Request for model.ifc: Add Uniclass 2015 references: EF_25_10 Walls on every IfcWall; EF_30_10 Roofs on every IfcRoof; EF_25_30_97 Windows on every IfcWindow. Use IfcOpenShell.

First a look at what the model holds.

```python
import ifcopenshell

model = ifcopenshell.open("model.ifc")
print(model.schema)
print("classifications:", [c.Name for c in model.by_type("IfcClassification")])
for ifc_class in ("IfcDoor", "IfcRoof", "IfcStair", "IfcWall", "IfcWindow"):
    print(ifc_class, len(model.by_type(ifc_class)))
```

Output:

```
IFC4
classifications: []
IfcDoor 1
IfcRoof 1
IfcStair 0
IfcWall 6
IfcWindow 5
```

```python
import ifcopenshell
import ifcopenshell.api.classification

model = ifcopenshell.open("model.ifc")

system = ifcopenshell.api.classification.add_classification(model, classification="Uniclass 2015")

codes = {
    "IfcWall": ("EF_25_10", "Walls"),
    "IfcRoof": ("EF_30_10", "Roofs"),
    "IfcWindow": ("EF_25_30_97", "Windows"),
}
for ifc_class, (code, name) in codes.items():
    products = model.by_type(ifc_class)
    ifcopenshell.api.classification.add_reference(
        model, products=products, classification=system, identification=code, name=name
    )
    print(code, len(products))

model.write("model_edited.ifc")
```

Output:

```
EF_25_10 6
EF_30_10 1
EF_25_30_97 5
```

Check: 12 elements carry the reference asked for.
